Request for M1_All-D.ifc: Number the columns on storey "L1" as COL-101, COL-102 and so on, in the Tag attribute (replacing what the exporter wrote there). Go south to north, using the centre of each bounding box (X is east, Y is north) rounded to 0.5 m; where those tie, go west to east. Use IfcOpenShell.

First a look at what the model holds.

```python
import ifcopenshell
import ifcopenshell.util.element
import ifcopenshell.util.placement

model = ifcopenshell.open("M1_All-D.ifc")
print(model.schema)
storey = next(s for s in model.by_type("IfcBuildingStorey") if s.Name == "L1")
columns = [e for e in ifcopenshell.util.element.get_decomposition(storey) if e.is_a("IfcColumn")]
for e in sorted(columns, key=lambda e: e.id()):
    origin = ifcopenshell.util.placement.get_local_placement(e.ObjectPlacement)[:3, 3]
    print(e.id(), e.Tag, e.Name, origin.round(2) + 0.0, sep=" | ")
```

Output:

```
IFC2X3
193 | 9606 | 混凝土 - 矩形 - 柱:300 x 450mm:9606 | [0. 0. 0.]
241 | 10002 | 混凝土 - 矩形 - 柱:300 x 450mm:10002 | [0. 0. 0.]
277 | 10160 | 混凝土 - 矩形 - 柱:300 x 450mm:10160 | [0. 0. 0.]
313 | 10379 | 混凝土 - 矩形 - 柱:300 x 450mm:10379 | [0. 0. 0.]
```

```python
import ifcopenshell
import ifcopenshell.geom
import ifcopenshell.util.element
import ifcopenshell.util.shape

model = ifcopenshell.open("M1_All-D.ifc")
settings = ifcopenshell.geom.settings()
settings.set("use-world-coords", True)


def centre(element):
    shape = ifcopenshell.geom.create_shape(settings, element)
    return ifcopenshell.util.shape.get_bbox_centroid(shape.geometry)


storey = next(s for s in model.by_type("IfcBuildingStorey") if s.Name == "L1")
columns = [e for e in ifcopenshell.util.element.get_decomposition(storey) if e.is_a("IfcColumn")]

# Insertion points can sit at a corner or the storey origin, so sort by the geometry (in metres).
centres = {e: centre(e) for e in columns}
columns.sort(key=lambda e: (round(centres[e][1] / 0.5), centres[e][0]))

for i, e in enumerate(columns, start=1):
    number = f"COL-1{i:02d}"
    e.Tag = number
    print(e.id(), number)

model.write("M1_All-D_v2.ifc")
```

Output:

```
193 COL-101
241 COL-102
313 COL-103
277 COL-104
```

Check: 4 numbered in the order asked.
